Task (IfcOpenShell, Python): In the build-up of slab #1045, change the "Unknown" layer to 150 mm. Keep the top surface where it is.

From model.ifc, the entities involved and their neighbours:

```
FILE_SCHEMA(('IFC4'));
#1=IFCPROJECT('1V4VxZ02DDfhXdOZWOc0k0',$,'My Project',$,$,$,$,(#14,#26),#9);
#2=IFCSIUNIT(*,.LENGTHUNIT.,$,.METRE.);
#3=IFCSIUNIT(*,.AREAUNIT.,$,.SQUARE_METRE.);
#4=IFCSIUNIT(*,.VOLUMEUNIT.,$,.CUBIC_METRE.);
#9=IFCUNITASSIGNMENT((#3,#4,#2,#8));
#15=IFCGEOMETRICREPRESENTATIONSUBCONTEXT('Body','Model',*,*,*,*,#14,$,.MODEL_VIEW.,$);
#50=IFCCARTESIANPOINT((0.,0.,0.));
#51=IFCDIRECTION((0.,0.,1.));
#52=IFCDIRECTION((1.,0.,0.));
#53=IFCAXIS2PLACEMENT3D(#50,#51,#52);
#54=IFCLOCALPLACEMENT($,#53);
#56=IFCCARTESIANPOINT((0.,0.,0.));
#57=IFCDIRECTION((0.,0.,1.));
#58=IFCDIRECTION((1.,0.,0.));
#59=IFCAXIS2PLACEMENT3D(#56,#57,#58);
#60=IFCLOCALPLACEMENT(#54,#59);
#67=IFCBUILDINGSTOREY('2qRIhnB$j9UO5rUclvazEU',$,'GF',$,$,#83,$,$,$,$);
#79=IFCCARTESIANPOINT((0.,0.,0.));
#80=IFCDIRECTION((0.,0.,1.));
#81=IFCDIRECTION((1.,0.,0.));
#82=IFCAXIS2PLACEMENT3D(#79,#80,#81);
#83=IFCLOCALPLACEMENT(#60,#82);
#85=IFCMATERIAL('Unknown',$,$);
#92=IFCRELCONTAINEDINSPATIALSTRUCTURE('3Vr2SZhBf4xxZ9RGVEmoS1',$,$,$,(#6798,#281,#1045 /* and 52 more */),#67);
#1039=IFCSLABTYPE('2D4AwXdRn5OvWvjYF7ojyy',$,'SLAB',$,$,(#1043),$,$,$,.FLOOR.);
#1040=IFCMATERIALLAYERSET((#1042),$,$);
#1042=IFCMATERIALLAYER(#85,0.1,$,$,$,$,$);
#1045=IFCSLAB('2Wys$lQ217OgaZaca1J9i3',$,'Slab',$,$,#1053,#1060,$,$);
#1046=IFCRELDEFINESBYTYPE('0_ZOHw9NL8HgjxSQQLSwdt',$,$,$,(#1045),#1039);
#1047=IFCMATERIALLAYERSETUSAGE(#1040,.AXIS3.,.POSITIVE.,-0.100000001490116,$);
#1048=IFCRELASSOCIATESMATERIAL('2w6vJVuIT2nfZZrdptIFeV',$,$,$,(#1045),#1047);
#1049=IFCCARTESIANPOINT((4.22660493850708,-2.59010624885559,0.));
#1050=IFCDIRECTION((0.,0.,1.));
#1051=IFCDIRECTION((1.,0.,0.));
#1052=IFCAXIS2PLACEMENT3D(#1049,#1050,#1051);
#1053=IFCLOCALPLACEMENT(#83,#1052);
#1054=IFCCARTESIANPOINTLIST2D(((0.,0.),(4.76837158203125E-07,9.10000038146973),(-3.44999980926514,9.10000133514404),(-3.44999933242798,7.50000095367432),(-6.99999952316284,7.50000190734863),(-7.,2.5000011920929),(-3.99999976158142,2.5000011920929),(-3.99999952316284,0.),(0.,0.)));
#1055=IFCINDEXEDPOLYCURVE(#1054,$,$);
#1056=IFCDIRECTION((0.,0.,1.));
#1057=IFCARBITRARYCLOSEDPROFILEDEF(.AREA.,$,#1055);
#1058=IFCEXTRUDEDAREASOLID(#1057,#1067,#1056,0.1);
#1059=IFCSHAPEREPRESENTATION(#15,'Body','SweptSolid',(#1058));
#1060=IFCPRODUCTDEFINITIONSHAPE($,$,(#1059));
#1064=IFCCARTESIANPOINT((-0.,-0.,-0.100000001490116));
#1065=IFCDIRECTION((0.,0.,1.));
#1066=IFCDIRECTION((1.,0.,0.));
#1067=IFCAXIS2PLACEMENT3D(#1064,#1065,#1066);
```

```python
import ifcopenshell
import ifcopenshell.util.element
import ifcopenshell.util.representation

model = ifcopenshell.open("model.ifc")

layer_set = model.by_id(1040)
layer = next(l for l in layer_set.MaterialLayers if l.Material and l.Material.Name == "Unknown")
change = 0.15 - layer.LayerThickness
layer.LayerThickness += change

# Geometry does not follow the layer set by itself.
slabs = [e for e in ifcopenshell.util.element.get_elements_by_material(model, layer_set) if e.is_a("IfcSlab")]
for slab in sorted(slabs, key=lambda e: e.id()):
    body = ifcopenshell.util.representation.get_representation(slab, "Model", "Body")
    solid = body.Items[0]
    old_depth = solid.Depth
    solid.Depth += change
    # Extruded upwards: lower the start of the extrusion so the top stays.
    x, y, z = solid.Position.Location.Coordinates
    solid.Position.Location = model.createIfcCartesianPoint((x, y, z - change))
    print(slab.id(), f"{old_depth:g} -> {solid.Depth:g}")

# The layers are counted up from the underside, which has moved.
for usage in {ifcopenshell.util.element.get_material(slab) for slab in slabs}:
    usage.OffsetFromReferenceLine -= change

model.write("model_rev.ifc")
```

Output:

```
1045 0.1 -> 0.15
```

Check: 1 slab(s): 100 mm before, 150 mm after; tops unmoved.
